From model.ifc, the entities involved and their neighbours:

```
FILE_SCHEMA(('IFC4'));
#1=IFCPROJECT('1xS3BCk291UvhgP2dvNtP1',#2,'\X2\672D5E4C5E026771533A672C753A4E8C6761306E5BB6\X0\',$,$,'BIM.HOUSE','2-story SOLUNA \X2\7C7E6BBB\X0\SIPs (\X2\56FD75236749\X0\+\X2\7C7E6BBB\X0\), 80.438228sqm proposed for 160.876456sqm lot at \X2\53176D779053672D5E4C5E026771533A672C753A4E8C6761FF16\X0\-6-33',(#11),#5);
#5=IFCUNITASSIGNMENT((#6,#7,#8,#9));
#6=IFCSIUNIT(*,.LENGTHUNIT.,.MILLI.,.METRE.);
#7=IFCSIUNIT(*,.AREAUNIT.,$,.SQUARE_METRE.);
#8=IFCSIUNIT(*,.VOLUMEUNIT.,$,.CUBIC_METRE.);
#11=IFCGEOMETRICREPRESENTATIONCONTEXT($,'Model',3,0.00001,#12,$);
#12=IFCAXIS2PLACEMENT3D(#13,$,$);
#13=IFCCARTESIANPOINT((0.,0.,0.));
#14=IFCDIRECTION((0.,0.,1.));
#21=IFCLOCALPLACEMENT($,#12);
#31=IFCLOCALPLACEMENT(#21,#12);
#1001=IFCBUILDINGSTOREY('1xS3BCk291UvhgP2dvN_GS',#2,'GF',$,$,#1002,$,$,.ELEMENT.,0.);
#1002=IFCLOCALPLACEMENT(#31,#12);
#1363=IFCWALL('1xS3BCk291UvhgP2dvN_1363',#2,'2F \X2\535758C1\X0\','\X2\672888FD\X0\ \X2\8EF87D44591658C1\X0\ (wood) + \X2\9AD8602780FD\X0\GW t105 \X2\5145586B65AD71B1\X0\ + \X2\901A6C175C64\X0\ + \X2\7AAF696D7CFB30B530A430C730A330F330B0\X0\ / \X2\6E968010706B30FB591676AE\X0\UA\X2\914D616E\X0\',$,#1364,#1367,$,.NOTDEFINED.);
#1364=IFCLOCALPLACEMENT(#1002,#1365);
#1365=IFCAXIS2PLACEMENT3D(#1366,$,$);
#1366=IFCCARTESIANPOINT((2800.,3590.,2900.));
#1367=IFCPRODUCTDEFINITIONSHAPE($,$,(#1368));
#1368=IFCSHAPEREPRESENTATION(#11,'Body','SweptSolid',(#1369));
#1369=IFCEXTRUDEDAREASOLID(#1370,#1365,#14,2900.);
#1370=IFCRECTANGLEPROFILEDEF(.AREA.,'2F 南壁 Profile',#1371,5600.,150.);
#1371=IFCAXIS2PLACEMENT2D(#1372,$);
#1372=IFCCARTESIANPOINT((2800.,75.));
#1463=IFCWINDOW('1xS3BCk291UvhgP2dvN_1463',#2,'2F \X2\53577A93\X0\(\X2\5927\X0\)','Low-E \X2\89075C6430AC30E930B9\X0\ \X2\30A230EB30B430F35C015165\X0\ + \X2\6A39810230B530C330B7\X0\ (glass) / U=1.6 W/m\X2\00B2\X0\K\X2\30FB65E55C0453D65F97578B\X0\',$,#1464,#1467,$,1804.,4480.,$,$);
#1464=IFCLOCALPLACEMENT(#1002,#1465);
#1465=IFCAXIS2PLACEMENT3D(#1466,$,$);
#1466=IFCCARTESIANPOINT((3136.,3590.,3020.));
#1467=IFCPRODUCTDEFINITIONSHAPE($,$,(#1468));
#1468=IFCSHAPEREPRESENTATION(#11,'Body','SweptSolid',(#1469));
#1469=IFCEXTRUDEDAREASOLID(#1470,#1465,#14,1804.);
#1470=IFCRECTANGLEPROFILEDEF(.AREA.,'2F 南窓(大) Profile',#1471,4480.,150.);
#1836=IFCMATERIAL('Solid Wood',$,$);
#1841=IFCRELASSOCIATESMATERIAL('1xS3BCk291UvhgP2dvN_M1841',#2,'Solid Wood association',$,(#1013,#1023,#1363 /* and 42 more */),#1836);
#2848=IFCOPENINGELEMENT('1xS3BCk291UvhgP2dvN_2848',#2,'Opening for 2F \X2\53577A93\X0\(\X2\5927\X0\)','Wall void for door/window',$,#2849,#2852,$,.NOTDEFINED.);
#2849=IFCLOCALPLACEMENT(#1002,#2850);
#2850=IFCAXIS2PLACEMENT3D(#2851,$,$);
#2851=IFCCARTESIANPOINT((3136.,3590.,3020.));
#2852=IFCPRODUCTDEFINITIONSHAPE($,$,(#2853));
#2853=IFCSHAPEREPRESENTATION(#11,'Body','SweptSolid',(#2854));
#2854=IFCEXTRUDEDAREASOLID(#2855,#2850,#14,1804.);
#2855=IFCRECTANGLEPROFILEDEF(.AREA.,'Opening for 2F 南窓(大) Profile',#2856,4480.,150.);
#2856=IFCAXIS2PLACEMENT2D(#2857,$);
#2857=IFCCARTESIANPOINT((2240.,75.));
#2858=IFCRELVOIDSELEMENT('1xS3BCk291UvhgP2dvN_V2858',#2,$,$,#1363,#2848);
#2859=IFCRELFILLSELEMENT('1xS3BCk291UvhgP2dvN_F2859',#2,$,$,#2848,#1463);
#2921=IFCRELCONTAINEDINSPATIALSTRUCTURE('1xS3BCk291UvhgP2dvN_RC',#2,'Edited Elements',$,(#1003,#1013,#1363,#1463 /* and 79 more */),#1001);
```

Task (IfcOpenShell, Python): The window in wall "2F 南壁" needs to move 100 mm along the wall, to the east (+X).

```python
import ifcopenshell
import ifcopenshell.api.geometry
import ifcopenshell.util.placement

model = ifcopenshell.open("model.ifc")

window = model.by_guid("1xS3BCk291UvhgP2dvN_1463")
opening = window.FillsVoids[0].RelatingOpeningElement
wall = opening.VoidsElements[0].RelatingBuildingElement

wall_matrix = ifcopenshell.util.placement.get_local_placement(wall.ObjectPlacement)
shift = wall_matrix[:3, 0] * 100.0
before = ifcopenshell.util.placement.get_local_placement(window.ObjectPlacement)[:3, 3].copy()

# The window is not placed relative to its opening, so move both.
for product in (opening, window):
    matrix = ifcopenshell.util.placement.get_local_placement(product.ObjectPlacement)
    matrix[:3, 3] += shift
    ifcopenshell.api.geometry.edit_object_placement(model, product=product, matrix=matrix, is_si=False)

after = ifcopenshell.util.placement.get_local_placement(window.ObjectPlacement)[:3, 3]
print("window moved by", (after - before).round(3) + 0.0)

model.write("model-out.ifc")
```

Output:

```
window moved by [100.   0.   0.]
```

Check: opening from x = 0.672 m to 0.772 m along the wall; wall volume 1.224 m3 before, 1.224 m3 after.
